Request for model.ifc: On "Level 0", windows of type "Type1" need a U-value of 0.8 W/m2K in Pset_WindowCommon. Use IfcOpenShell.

First a look at what the model holds.

```python
import ifcopenshell
import ifcopenshell.util.element

model = ifcopenshell.open("model.ifc")
print(model.schema)
storey = next(s for s in model.by_type("IfcBuildingStorey") if s.Name == "Level 0")
windows = [e for e in ifcopenshell.util.element.get_decomposition(storey) if e.is_a("IfcWindow")]
seen = {}
for e in windows:
    element_type = ifcopenshell.util.element.get_type(e)
    key = (element_type.Name if element_type != e and element_type else None, ifcopenshell.util.element.get_pset(e, "Pset_WindowCommon", "ThermalTransmittance"))
    seen[key] = seen.get(key, 0) + 1
for (name, value), count in sorted(seen.items(), key=str):
    print(count, "x", name, "|", value)
```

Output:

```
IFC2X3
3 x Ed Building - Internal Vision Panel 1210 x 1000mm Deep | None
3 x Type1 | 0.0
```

```python
import ifcopenshell
import ifcopenshell.api.pset
import ifcopenshell.util.element

model = ifcopenshell.open("model.ifc")

storey = next(s for s in model.by_type("IfcBuildingStorey") if s.Name == "Level 0")
windows = [e for e in ifcopenshell.util.element.get_decomposition(storey) if e.is_a("IfcWindow")]

count = 0
for e in windows:
    element_type = ifcopenshell.util.element.get_type(e)
    if element_type in (None, e) or element_type.Name != "Type1":
        continue
    # add_pset returns the element's existing set when there is one.
    pset = ifcopenshell.api.pset.add_pset(model, product=e, name="Pset_WindowCommon")
    ifcopenshell.api.pset.edit_pset(model, pset=pset, properties={"ThermalTransmittance": 0.8})
    count += 1

print(count, "windows updated")

model.write("model-out.ifc")
```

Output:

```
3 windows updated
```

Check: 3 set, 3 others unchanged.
